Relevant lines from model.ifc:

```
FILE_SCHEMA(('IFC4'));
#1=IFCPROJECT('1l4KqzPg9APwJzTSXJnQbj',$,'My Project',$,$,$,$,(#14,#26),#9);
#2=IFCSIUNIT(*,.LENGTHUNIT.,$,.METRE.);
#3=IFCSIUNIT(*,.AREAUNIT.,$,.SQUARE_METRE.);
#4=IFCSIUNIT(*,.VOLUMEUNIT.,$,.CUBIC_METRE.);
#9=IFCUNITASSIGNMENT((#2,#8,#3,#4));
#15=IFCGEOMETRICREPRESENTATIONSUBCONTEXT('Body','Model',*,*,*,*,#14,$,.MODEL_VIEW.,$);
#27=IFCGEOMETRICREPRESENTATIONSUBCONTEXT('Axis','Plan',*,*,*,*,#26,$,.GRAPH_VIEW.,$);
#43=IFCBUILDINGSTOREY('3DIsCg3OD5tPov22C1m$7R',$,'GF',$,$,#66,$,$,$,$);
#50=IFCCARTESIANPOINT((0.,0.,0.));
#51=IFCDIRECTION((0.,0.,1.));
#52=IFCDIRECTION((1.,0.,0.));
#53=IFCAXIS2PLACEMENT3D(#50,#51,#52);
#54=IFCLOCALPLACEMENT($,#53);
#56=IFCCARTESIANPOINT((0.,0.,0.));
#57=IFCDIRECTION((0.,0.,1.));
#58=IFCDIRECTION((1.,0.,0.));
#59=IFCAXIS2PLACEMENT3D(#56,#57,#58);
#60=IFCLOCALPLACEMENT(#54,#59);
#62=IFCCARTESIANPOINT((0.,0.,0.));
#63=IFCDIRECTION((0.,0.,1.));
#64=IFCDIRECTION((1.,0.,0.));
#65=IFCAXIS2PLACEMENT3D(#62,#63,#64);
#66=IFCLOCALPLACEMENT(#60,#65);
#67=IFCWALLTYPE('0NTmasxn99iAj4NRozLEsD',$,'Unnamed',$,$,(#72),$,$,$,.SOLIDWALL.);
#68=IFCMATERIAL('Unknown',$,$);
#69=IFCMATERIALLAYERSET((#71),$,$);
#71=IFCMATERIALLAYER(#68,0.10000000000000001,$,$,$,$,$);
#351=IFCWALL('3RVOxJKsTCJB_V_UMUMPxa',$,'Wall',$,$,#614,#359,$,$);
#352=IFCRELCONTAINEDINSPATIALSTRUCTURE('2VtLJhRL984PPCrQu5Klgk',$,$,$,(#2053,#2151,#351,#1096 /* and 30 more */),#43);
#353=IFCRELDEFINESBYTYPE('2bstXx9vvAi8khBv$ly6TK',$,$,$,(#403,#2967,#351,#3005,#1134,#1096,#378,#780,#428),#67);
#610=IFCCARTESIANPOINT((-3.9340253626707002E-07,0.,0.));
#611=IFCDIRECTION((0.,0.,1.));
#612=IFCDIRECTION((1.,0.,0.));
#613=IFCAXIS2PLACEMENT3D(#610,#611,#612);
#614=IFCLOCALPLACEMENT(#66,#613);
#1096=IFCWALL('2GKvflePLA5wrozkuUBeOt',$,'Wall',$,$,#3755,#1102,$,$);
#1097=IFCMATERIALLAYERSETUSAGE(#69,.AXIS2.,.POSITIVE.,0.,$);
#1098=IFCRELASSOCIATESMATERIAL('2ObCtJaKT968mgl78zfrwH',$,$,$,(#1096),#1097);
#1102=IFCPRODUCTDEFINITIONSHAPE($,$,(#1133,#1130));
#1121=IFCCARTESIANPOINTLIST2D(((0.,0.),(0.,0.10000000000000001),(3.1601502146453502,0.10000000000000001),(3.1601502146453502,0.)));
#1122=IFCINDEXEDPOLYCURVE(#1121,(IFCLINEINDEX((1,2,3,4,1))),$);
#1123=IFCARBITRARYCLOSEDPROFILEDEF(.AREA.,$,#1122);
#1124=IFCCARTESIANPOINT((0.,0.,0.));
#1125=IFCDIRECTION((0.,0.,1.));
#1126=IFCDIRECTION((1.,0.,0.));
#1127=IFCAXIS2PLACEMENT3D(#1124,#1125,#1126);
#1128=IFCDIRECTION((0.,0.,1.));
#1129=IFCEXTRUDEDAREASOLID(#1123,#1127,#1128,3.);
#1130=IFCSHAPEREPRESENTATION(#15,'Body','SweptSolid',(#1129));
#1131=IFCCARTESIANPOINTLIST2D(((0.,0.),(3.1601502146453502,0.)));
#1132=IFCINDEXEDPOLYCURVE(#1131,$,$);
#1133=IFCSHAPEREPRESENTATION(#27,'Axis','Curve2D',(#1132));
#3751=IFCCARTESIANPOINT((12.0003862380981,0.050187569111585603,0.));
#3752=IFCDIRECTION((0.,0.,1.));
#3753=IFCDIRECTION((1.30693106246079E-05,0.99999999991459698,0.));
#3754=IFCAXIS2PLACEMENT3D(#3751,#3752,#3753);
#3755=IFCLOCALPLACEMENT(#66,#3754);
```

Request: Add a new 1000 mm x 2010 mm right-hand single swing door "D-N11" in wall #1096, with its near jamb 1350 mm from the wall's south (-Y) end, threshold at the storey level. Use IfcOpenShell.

```python
import numpy as np
import ifcopenshell
import ifcopenshell.api.feature
import ifcopenshell.api.geometry
import ifcopenshell.api.root
import ifcopenshell.api.spatial
import ifcopenshell.geom
import ifcopenshell.util.element
import ifcopenshell.util.placement
import ifcopenshell.util.representation
import ifcopenshell.util.shape
import ifcopenshell.util.unit

model = ifcopenshell.open("model.ifc")
unit_scale = ifcopenshell.util.unit.calculate_unit_scale(model)
settings = ifcopenshell.geom.settings()


def volume(element):
    """Net volume in cubic metres, openings subtracted."""
    shape = ifcopenshell.geom.create_shape(settings, element)
    return ifcopenshell.util.shape.get_volume(shape.geometry)


wall = model.by_guid("2GKvflePLA5wrozkuUBeOt")
storey = ifcopenshell.util.element.get_container(wall, ifc_class="IfcBuildingStorey")
context = ifcopenshell.util.representation.get_context(model, "Model", "Body", "MODEL_VIEW")
before = volume(wall)

width, height, from_end, sill = 1, 2.01, 1.35, 0.0  # metres

# The wall runs along its own X axis, and the end named is its -X end.
wall_shape = ifcopenshell.geom.create_shape(settings, wall)
x, y, z = ifcopenshell.util.shape.get_vertices(wall_shape.geometry).T
start = x.min() + from_end
face, thickness = float(y.min()), float(y.max() - y.min())
wall_matrix = ifcopenshell.util.placement.get_local_placement(wall.ObjectPlacement)
level = ifcopenshell.util.placement.get_local_placement(storey.ObjectPlacement)[2, 3]


def in_wall(x, y):
    """Placement at x, y metres in the wall's axes, at sill height."""
    matrix = wall_matrix.copy()
    matrix[:, 3] = wall_matrix @ np.array([x / unit_scale, y / unit_scale, 0.0, 1.0])
    matrix[2, 3] = level + sill / unit_scale
    return matrix


# Opening: a box that overshoots both wall faces by 50 mm.
opening = ifcopenshell.api.root.create_entity(model, ifc_class="IfcOpeningElement", predefined_type="OPENING")
box = ifcopenshell.api.geometry.add_wall_representation(
    model, context=context, length=width, height=height, thickness=thickness + 0.1
)
ifcopenshell.api.geometry.assign_representation(model, product=opening, representation=box)
ifcopenshell.api.geometry.edit_object_placement(model, product=opening, matrix=in_wall(start, face - 0.05), is_si=False)
ifcopenshell.api.feature.add_feature(model, feature=opening, element=wall)

door = ifcopenshell.api.root.create_entity(model, ifc_class="IfcDoor", name="D-N11", predefined_type="DOOR")
door.OverallWidth, door.OverallHeight = width / unit_scale, height / unit_scale
door.OperationType = "SINGLE_SWING_RIGHT"
body = ifcopenshell.api.geometry.add_door_representation(
    model,
    context=context,
    overall_width=door.OverallWidth,
    overall_height=door.OverallHeight,
    operation_type="SINGLE_SWING_RIGHT",
    lining_properties={"LiningDepth": thickness / unit_scale, "ThresholdDepth": thickness / unit_scale},
)
ifcopenshell.api.geometry.assign_representation(model, product=door, representation=body)
ifcopenshell.api.spatial.assign_container(model, products=[door], relating_structure=storey)
ifcopenshell.api.feature.add_filling(model, opening=opening, element=door)

# The lining spans the wall, so the door starts at the wall face.
ifcopenshell.api.geometry.edit_object_placement(model, product=door, matrix=in_wall(start, face), is_si=False)

after = volume(wall)

print(f"wall volume {before:.3f} -> {after:.3f} m3")

model.write("model-out.ifc")
```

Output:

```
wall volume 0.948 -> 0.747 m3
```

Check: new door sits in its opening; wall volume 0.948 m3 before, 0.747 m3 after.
